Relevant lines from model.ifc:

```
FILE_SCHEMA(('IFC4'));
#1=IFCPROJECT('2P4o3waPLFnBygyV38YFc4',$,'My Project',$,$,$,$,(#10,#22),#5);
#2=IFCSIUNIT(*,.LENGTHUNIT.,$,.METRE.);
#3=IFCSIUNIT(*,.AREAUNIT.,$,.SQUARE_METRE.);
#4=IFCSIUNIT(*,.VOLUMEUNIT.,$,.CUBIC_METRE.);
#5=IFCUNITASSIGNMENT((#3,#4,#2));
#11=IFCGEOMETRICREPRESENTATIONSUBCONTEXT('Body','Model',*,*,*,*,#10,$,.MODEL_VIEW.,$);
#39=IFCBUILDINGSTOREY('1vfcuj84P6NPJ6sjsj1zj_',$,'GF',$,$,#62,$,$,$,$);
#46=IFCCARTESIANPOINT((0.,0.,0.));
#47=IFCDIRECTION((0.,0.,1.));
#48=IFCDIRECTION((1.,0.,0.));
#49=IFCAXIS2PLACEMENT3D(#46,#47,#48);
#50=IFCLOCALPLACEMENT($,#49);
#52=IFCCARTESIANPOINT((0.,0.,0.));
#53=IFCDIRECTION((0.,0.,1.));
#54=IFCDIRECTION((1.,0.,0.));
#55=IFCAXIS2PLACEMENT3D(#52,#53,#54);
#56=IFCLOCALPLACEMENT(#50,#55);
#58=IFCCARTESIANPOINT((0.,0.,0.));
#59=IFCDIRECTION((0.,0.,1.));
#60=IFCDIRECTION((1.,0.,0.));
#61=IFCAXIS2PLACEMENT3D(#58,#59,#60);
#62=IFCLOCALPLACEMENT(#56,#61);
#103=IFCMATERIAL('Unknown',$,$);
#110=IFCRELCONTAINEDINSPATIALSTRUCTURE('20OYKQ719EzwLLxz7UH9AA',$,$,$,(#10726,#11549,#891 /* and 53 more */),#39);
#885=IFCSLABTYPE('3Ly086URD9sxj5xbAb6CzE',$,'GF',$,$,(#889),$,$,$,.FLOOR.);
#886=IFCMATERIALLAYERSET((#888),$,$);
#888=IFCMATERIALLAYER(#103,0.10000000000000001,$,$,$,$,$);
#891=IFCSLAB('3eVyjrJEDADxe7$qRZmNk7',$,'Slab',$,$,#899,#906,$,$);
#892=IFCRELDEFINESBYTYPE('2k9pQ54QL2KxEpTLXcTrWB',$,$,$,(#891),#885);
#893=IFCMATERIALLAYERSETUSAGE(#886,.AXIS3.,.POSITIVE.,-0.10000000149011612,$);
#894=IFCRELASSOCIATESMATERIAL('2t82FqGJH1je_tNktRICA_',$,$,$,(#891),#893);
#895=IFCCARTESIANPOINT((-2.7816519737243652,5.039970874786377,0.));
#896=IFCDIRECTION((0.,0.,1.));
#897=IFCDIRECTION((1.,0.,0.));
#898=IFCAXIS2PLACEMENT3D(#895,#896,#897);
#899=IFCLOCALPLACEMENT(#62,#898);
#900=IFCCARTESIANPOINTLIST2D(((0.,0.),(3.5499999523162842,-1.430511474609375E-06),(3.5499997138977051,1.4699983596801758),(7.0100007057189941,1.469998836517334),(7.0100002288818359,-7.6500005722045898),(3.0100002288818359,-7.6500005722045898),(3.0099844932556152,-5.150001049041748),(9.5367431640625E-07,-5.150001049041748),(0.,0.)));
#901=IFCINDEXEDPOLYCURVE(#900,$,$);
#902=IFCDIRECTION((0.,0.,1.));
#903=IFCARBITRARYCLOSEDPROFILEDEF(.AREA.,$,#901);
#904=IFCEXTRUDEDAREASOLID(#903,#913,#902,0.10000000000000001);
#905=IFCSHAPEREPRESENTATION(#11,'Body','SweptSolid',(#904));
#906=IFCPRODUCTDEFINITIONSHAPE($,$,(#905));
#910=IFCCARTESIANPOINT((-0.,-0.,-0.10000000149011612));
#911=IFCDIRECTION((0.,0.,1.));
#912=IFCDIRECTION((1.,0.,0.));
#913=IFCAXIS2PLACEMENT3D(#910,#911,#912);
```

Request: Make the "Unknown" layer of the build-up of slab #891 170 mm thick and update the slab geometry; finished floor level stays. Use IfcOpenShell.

```python
import ifcopenshell
import ifcopenshell.util.element
import ifcopenshell.util.representation
import ifcopenshell.util.unit

model = ifcopenshell.open("model.ifc")
unit_scale = ifcopenshell.util.unit.calculate_unit_scale(model)

layer_set = model.by_id(886)
layer = next(l for l in layer_set.MaterialLayers if l.Material and l.Material.Name == "Unknown")
change = 0.17 / unit_scale - layer.LayerThickness
layer.LayerThickness += change

# Geometry does not follow the layer set by itself.
slabs = [e for e in ifcopenshell.util.element.get_elements_by_material(model, layer_set) if e.is_a("IfcSlab")]
for slab in sorted(slabs, key=lambda e: e.id()):
    body = ifcopenshell.util.representation.get_representation(slab, "Model", "Body")
    solid = body.Items[0]
    old_depth = solid.Depth
    solid.Depth += change
    # Extruded upwards: lower the start of the extrusion so the top stays.
    x, y, z = solid.Position.Location.Coordinates
    solid.Position.Location = model.createIfcCartesianPoint((x, y, z - change))
    print(slab.id(), f"{old_depth:g} -> {solid.Depth:g}")

# The layers are counted up from the underside, which has moved.
for usage in {ifcopenshell.util.element.get_material(slab) for slab in slabs}:
    usage.OffsetFromReferenceLine -= change

model.write("model_updated.ifc")
```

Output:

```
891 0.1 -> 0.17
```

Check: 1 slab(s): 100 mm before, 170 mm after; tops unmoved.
